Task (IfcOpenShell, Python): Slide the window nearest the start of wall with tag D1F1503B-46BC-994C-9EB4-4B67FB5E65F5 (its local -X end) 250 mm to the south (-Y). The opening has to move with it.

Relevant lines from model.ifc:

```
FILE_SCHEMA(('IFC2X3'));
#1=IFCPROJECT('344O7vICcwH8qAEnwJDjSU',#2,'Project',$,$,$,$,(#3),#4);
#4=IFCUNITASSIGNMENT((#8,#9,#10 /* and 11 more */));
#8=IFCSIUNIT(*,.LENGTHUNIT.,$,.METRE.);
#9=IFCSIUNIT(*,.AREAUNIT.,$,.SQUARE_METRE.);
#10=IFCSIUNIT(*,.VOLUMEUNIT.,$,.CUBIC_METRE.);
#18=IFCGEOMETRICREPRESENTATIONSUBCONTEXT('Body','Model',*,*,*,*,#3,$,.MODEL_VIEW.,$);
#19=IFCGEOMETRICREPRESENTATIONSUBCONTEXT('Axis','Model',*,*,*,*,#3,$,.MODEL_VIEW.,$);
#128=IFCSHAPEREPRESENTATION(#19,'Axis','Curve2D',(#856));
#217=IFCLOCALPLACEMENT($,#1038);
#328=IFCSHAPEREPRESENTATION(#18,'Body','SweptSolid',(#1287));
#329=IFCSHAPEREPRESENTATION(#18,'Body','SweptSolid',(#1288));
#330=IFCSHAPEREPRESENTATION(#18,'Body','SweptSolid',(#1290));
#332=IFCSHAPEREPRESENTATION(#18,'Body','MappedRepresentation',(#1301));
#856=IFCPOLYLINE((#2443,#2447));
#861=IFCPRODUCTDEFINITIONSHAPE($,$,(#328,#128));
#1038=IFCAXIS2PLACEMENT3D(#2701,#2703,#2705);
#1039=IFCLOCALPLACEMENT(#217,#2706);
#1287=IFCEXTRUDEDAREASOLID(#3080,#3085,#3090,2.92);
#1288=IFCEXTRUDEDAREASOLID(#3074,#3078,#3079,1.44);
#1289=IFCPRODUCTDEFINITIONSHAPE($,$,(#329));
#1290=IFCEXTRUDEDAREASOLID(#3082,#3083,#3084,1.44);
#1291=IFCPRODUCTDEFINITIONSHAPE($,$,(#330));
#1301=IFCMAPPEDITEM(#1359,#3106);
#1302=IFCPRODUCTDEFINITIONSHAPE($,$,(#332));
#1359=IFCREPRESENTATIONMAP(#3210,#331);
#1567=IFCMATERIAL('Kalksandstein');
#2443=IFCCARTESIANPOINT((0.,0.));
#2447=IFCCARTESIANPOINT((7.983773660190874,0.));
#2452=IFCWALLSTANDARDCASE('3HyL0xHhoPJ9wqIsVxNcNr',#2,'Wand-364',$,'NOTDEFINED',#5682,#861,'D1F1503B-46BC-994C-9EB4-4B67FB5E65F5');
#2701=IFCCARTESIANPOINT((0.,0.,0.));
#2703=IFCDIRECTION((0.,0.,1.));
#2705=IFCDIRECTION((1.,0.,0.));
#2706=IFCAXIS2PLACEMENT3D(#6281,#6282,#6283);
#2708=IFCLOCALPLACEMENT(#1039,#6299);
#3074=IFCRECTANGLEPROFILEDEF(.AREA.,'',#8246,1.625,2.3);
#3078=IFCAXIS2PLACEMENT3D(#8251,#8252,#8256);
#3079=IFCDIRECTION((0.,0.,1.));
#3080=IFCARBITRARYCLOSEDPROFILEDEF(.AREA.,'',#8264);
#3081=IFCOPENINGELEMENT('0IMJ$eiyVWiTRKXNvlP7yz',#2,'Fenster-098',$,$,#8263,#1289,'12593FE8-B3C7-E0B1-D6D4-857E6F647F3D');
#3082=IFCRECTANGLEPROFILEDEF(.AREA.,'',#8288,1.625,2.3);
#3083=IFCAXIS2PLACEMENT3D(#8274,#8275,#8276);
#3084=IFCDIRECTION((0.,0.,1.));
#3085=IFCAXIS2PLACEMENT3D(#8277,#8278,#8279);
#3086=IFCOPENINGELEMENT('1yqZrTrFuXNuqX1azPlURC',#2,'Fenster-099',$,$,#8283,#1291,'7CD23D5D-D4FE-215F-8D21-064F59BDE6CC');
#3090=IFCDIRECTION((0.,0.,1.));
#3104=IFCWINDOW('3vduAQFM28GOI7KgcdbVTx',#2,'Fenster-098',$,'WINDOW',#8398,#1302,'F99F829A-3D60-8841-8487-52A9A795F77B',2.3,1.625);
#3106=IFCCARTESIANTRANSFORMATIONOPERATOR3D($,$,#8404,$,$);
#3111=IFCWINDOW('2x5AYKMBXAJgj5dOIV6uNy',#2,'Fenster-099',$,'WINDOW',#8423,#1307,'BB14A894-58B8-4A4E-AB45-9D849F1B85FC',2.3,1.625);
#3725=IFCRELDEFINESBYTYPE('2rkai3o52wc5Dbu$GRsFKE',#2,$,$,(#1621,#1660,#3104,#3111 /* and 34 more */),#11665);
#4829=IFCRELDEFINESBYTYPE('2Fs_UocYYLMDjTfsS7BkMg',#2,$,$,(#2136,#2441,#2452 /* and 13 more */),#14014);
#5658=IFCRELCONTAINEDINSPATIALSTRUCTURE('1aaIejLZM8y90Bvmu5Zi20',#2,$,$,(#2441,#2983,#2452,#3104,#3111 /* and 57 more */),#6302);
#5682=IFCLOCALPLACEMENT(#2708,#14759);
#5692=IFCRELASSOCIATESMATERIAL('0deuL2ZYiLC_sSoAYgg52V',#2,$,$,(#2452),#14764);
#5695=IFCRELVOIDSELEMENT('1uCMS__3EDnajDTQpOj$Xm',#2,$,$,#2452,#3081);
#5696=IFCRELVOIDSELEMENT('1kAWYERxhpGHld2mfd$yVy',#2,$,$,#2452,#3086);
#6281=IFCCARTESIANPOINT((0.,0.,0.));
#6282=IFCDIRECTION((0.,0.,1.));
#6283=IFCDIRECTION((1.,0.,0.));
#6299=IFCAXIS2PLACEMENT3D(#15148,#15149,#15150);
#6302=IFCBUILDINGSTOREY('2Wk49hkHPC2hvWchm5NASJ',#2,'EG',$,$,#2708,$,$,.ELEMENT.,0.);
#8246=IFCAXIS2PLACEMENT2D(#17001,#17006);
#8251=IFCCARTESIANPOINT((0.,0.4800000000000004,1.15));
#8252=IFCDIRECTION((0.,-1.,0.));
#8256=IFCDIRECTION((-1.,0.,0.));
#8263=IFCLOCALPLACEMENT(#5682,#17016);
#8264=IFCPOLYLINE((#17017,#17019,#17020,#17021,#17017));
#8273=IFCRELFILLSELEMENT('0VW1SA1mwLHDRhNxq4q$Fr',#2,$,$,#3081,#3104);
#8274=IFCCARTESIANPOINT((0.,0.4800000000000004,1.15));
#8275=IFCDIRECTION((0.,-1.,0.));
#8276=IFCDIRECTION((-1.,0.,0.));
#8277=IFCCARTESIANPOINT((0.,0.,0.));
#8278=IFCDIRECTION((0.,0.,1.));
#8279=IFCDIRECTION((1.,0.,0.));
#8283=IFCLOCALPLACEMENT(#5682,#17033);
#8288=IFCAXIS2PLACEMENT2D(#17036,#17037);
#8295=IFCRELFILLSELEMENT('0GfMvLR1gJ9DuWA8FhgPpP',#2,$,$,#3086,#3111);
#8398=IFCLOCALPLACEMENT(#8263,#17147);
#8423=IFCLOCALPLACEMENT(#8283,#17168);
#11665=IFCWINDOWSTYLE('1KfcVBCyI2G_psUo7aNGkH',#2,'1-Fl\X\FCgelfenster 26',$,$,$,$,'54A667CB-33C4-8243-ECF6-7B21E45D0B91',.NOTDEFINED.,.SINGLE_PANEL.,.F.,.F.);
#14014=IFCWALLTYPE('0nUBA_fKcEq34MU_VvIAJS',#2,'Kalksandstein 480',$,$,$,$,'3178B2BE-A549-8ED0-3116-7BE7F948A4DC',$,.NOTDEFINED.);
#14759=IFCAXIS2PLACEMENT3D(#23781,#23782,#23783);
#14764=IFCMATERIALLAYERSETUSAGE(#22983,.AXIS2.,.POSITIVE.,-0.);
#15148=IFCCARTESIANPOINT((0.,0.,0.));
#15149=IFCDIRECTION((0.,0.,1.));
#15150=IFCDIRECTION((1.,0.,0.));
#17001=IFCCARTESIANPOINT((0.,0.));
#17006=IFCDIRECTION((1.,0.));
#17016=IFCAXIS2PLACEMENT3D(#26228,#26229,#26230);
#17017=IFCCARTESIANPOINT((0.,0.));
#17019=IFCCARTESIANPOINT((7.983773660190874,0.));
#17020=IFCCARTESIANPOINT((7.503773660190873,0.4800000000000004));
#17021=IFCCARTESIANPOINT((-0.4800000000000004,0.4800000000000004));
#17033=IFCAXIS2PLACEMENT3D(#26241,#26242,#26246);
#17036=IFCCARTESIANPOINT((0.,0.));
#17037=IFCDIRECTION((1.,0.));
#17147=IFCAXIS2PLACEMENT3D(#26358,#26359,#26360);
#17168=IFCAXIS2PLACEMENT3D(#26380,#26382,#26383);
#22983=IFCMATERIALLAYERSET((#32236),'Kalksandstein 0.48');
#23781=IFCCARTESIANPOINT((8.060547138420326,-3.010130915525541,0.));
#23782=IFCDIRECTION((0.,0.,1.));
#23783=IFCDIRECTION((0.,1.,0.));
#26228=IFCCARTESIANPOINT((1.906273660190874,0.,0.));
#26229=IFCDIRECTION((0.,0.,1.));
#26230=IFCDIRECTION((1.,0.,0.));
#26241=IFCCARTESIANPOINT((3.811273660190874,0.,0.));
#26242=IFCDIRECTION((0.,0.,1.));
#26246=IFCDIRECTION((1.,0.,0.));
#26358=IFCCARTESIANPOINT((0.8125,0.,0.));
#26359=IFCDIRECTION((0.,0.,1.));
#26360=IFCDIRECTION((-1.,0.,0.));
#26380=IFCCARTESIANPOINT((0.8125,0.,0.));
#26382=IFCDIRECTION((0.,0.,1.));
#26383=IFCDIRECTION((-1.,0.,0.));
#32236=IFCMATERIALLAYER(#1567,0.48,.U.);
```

```python
import ifcopenshell
import ifcopenshell.api.geometry
import ifcopenshell.util.placement
import ifcopenshell.util.unit

model = ifcopenshell.open("model.ifc")
unit_scale = ifcopenshell.util.unit.calculate_unit_scale(model)

window = model.by_id(3104)
opening = window.FillsVoids[0].RelatingOpeningElement
wall = opening.VoidsElements[0].RelatingBuildingElement

wall_matrix = ifcopenshell.util.placement.get_local_placement(wall.ObjectPlacement)
shift = wall_matrix[:3, 0] * -0.25 / unit_scale
before = ifcopenshell.util.placement.get_local_placement(window.ObjectPlacement)[:3, 3].copy()

# The window is placed relative to its opening, so it follows when the opening moves.
matrix = ifcopenshell.util.placement.get_local_placement(opening.ObjectPlacement)
matrix[:3, 3] += shift
ifcopenshell.api.geometry.edit_object_placement(
    model, product=opening, matrix=matrix, is_si=False, should_transform_children=True
)

after = ifcopenshell.util.placement.get_local_placement(window.ObjectPlacement)[:3, 3]
print("window moved by", (after - before).round(3) + 0.0)

model.write("model_edited.ifc")
```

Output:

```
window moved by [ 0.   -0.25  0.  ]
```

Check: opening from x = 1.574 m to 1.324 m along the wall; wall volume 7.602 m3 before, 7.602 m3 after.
